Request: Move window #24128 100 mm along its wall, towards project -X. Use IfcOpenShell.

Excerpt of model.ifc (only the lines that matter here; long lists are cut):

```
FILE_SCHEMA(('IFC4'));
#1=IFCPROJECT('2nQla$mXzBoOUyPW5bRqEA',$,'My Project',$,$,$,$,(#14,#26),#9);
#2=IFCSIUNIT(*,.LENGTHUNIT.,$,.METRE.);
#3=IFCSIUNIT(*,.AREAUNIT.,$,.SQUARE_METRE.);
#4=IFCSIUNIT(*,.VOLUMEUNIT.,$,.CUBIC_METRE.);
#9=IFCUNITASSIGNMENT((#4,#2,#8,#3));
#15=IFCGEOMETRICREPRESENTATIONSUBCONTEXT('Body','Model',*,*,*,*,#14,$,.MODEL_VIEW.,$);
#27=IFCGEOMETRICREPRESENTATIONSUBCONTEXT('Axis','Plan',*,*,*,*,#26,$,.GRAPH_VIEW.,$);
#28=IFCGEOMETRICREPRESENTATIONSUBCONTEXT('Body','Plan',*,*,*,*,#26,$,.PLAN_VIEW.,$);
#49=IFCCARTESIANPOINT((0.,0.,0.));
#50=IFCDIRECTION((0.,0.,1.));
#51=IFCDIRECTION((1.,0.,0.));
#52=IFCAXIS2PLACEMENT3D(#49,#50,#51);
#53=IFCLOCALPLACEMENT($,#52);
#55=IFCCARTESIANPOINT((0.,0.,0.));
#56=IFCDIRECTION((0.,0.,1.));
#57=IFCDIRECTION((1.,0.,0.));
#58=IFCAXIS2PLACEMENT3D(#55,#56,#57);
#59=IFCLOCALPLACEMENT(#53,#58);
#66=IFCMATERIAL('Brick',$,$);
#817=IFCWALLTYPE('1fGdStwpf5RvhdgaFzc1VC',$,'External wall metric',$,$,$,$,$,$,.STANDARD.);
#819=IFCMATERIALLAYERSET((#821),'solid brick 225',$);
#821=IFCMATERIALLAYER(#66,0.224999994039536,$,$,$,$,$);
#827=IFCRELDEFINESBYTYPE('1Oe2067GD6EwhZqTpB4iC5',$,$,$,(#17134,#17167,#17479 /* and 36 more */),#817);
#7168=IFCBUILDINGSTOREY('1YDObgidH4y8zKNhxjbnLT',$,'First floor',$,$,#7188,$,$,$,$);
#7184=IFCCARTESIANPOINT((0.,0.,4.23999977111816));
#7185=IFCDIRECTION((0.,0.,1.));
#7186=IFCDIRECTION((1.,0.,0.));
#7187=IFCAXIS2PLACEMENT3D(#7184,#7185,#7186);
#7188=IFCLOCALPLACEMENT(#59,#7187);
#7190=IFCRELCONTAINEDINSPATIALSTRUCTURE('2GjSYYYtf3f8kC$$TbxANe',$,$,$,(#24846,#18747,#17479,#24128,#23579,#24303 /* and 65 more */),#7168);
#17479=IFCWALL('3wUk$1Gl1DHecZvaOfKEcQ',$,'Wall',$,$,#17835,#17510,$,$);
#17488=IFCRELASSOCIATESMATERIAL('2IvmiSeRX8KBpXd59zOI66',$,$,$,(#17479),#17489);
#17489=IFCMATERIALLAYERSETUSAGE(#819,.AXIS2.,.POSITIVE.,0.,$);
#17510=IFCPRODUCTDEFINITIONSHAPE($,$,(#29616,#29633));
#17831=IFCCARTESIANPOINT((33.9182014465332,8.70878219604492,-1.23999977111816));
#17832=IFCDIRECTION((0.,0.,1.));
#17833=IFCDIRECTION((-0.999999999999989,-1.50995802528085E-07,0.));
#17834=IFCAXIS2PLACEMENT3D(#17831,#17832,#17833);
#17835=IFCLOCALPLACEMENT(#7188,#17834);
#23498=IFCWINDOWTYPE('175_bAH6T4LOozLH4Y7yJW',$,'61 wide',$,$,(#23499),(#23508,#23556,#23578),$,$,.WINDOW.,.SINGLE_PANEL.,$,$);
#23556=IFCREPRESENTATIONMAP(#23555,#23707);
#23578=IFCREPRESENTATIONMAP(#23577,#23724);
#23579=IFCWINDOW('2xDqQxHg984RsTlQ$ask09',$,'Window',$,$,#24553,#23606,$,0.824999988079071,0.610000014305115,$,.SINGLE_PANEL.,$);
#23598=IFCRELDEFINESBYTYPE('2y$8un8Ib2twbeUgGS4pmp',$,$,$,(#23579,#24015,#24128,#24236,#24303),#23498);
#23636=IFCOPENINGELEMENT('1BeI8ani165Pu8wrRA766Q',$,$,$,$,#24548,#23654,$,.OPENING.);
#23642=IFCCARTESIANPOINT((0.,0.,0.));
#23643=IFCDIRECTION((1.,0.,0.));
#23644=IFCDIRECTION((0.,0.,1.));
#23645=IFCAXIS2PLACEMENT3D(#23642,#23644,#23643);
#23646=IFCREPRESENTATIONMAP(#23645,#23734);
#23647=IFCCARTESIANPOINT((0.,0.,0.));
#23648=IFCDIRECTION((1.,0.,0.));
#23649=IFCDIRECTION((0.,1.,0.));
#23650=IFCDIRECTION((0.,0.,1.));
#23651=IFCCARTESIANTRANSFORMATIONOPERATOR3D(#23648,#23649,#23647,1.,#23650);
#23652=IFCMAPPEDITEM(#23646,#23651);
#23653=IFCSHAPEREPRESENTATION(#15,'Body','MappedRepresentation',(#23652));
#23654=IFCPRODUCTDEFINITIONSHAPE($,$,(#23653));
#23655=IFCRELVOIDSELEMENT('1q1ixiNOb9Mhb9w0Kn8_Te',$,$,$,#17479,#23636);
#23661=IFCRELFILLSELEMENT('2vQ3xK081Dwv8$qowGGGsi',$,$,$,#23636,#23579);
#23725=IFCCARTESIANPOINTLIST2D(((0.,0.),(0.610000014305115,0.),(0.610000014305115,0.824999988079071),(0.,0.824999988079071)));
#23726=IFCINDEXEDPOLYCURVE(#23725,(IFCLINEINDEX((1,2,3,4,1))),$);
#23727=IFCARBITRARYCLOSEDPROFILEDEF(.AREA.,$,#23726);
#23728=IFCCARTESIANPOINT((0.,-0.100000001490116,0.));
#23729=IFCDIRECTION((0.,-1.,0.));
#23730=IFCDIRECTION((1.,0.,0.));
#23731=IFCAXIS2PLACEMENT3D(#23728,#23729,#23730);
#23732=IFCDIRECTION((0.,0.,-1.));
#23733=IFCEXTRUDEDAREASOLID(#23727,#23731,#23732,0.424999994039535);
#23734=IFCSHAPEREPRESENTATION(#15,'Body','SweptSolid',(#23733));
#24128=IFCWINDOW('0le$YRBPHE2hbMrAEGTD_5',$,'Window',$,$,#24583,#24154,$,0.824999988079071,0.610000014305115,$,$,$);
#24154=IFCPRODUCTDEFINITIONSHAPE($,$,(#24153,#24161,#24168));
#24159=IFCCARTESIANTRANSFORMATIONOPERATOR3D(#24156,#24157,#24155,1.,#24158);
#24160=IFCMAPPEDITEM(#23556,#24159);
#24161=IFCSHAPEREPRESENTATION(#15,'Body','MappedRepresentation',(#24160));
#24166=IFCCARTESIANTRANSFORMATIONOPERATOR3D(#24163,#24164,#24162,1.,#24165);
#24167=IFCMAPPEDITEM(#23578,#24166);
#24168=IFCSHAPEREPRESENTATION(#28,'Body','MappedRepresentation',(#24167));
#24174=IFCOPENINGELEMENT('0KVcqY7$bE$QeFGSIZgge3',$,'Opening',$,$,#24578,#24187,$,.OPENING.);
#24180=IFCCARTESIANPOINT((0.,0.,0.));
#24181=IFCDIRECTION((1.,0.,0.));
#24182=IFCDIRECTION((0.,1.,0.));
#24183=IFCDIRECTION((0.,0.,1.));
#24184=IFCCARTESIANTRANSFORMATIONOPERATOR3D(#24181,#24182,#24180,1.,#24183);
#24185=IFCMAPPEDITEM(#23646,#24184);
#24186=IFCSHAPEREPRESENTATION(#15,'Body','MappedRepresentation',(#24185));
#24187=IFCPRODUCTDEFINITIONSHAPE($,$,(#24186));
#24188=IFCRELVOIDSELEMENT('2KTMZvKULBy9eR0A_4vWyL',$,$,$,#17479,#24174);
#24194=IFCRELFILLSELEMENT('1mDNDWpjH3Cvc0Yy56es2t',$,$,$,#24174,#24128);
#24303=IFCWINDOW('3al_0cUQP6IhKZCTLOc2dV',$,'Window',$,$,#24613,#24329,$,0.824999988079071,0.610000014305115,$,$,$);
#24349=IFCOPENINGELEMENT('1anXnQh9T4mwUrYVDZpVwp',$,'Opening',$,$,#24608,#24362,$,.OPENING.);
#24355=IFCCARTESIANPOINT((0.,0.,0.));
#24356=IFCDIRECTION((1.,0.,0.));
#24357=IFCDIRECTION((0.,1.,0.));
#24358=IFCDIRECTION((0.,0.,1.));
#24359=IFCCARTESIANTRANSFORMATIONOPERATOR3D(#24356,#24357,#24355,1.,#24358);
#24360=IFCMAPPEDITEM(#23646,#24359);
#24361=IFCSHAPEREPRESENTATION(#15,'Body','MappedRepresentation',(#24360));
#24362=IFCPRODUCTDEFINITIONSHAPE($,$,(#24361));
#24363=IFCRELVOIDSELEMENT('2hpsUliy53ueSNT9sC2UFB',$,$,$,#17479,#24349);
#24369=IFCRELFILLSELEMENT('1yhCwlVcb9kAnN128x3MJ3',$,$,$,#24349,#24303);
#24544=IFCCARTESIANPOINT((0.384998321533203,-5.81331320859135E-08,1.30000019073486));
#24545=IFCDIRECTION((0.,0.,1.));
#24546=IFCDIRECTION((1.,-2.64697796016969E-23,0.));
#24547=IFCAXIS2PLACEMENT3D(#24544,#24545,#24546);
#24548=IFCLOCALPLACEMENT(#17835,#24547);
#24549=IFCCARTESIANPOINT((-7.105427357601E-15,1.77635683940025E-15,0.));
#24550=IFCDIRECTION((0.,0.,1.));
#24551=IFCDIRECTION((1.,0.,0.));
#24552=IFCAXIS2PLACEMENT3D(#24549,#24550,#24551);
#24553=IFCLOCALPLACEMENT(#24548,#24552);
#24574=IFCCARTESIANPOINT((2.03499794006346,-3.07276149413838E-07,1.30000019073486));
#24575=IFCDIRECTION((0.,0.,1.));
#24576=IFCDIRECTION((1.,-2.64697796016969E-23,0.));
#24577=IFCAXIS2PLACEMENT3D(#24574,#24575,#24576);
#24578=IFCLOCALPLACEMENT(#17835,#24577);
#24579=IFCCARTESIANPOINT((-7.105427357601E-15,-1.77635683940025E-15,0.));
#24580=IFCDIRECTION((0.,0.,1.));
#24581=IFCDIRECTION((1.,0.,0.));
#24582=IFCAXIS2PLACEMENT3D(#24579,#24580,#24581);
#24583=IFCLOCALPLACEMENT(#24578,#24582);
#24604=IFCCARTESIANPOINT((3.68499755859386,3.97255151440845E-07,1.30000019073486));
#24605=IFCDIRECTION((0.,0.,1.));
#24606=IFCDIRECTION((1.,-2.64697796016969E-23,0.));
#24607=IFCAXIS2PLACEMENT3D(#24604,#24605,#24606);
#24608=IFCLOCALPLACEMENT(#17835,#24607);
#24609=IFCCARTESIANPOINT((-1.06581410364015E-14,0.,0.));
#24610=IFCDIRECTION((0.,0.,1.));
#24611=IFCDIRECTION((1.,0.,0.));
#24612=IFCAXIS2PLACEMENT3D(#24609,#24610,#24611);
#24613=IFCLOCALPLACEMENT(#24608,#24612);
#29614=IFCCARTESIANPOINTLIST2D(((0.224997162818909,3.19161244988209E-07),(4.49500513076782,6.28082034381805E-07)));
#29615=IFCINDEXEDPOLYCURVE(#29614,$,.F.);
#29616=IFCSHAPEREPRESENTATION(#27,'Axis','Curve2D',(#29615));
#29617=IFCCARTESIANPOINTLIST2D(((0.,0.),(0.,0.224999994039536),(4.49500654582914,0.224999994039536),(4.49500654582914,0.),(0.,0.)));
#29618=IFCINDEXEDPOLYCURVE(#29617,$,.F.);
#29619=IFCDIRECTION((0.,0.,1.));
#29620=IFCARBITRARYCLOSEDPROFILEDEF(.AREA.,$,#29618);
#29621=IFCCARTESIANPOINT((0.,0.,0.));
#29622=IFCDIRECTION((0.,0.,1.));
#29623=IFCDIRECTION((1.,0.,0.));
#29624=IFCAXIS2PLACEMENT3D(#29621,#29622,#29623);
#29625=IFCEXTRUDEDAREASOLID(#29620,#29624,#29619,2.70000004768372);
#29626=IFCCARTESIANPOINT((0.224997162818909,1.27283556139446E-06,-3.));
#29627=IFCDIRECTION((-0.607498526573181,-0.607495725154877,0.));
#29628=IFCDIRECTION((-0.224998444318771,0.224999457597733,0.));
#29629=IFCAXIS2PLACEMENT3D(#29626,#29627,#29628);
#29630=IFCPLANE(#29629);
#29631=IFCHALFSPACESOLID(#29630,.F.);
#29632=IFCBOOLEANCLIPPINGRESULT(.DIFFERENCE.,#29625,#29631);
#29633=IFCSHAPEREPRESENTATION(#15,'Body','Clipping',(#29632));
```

```python
import ifcopenshell
import ifcopenshell.api.geometry
import ifcopenshell.util.placement
import ifcopenshell.util.unit

model = ifcopenshell.open("model.ifc")
unit_scale = ifcopenshell.util.unit.calculate_unit_scale(model)

window = model.by_guid("0le$YRBPHE2hbMrAEGTD_5")
opening = window.FillsVoids[0].RelatingOpeningElement
wall = opening.VoidsElements[0].RelatingBuildingElement

wall_matrix = ifcopenshell.util.placement.get_local_placement(wall.ObjectPlacement)
shift = wall_matrix[:3, 0] * 0.1 / unit_scale
before = ifcopenshell.util.placement.get_local_placement(window.ObjectPlacement)[:3, 3].copy()

# The window is placed relative to its opening, so it follows when the opening moves.
matrix = ifcopenshell.util.placement.get_local_placement(opening.ObjectPlacement)
matrix[:3, 3] += shift
ifcopenshell.api.geometry.edit_object_placement(
    model, product=opening, matrix=matrix, is_si=False, should_transform_children=True
)

after = ifcopenshell.util.placement.get_local_placement(window.ObjectPlacement)[:3, 3]
print("window moved by", (after - before).round(3) + 0.0)

model.write("model_v2.ifc")
```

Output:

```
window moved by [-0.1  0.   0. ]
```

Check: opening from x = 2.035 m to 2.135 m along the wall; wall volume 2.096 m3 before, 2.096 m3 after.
